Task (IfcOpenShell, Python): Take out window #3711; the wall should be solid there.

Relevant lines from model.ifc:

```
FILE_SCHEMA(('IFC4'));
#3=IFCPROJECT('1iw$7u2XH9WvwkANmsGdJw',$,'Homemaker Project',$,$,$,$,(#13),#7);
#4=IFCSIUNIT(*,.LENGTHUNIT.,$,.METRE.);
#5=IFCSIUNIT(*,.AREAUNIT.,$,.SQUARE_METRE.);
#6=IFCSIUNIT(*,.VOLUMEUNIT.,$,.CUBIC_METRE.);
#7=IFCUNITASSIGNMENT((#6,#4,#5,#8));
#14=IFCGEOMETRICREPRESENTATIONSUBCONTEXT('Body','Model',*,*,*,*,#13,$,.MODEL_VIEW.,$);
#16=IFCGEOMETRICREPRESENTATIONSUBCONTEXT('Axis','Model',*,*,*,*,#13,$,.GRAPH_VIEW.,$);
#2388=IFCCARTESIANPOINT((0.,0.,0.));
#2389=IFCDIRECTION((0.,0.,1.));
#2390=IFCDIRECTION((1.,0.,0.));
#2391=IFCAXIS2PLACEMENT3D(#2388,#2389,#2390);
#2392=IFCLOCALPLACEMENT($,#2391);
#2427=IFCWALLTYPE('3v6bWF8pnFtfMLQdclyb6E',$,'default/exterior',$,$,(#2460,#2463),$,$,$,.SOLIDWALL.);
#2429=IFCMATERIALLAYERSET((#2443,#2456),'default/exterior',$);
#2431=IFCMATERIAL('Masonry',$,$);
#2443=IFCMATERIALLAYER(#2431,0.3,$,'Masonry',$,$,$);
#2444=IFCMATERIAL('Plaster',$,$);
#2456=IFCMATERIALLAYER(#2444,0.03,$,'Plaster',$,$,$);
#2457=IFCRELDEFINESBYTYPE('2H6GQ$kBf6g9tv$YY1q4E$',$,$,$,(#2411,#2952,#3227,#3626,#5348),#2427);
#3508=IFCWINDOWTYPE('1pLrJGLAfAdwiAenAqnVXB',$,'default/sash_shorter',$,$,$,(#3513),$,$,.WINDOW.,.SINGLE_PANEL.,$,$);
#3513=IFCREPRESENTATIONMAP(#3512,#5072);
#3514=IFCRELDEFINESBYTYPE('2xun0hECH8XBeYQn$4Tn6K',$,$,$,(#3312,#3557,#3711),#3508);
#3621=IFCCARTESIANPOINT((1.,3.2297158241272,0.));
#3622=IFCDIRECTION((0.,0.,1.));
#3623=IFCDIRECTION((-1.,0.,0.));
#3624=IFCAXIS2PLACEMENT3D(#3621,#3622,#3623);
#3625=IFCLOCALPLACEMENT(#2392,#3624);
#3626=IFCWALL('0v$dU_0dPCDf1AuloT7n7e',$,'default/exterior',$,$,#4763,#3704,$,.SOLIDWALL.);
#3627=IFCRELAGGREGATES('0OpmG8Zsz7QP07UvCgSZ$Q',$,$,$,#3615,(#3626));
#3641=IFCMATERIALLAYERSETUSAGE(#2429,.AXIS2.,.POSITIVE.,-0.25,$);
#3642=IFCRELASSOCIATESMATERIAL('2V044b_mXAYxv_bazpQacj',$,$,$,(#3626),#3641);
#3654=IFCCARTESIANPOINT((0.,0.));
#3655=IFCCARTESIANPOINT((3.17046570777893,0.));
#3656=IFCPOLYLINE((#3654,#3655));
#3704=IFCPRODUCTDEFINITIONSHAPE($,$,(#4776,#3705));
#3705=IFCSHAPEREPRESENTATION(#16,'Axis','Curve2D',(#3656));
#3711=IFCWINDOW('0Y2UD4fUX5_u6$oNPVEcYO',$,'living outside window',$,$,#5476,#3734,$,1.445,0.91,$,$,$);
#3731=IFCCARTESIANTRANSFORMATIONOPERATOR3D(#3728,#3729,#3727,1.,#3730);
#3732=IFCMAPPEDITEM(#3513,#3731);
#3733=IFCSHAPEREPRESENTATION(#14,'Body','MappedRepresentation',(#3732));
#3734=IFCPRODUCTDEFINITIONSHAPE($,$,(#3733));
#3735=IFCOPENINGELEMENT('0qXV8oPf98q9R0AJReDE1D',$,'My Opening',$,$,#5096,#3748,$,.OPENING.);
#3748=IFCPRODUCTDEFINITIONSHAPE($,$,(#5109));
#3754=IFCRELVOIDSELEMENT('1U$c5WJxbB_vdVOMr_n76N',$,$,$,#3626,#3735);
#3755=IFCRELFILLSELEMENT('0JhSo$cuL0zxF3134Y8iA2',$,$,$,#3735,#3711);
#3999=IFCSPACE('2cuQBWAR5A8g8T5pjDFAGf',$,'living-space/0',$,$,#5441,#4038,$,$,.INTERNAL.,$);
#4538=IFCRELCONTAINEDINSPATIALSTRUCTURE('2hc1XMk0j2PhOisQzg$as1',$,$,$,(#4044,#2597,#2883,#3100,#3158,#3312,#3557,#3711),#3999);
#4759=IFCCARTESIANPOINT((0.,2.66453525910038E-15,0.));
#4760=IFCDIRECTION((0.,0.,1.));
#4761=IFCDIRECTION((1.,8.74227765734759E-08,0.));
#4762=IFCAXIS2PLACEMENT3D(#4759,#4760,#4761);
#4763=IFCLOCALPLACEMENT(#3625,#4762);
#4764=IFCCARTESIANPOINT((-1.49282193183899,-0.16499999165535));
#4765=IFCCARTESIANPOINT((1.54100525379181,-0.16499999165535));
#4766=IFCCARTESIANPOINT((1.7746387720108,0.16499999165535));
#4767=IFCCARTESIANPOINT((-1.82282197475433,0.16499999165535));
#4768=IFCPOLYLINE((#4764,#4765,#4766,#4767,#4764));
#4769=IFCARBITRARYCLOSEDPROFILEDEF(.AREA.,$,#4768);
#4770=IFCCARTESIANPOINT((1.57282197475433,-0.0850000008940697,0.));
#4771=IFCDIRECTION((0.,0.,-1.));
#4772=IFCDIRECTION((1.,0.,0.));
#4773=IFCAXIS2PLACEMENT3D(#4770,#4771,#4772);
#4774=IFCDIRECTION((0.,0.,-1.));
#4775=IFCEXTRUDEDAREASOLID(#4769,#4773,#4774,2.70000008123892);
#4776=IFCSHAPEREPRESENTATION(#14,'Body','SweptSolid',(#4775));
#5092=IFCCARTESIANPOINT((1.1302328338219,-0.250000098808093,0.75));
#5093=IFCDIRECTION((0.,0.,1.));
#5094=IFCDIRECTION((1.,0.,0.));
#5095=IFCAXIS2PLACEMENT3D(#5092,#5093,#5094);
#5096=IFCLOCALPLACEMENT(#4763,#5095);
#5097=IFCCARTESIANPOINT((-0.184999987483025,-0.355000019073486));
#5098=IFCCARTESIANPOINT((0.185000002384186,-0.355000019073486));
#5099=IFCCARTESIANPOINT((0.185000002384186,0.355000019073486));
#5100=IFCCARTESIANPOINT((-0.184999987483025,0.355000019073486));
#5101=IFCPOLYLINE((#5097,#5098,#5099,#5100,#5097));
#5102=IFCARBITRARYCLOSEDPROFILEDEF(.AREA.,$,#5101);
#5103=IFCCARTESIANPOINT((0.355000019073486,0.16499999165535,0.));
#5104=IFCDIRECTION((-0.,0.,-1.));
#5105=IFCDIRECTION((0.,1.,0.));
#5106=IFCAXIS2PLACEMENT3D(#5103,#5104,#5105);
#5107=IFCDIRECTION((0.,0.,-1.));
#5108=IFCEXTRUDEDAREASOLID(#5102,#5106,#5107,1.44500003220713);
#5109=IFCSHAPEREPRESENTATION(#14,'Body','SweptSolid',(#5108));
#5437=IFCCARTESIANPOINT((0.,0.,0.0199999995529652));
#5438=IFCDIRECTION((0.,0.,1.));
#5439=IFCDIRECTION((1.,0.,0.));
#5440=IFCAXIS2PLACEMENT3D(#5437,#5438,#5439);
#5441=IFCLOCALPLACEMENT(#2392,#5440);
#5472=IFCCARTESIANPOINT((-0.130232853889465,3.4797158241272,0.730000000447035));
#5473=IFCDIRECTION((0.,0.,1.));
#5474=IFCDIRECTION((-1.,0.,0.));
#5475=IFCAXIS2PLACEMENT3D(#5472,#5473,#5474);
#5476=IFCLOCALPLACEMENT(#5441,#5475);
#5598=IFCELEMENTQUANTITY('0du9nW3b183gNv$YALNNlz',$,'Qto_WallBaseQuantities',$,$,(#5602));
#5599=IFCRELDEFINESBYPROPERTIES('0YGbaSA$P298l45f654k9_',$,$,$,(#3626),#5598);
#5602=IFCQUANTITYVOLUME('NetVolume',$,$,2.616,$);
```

```python
import ifcopenshell
import ifcopenshell.api.feature
import ifcopenshell.api.pset
import ifcopenshell.api.root
import ifcopenshell.geom
import ifcopenshell.util.element
import ifcopenshell.util.shape
import ifcopenshell.util.unit

model = ifcopenshell.open("model.ifc")
volume_scale = ifcopenshell.util.unit.calculate_unit_scale(model, "VOLUMEUNIT")
settings = ifcopenshell.geom.settings()


def volume(element):
    """Net volume in cubic metres, openings subtracted."""
    shape = ifcopenshell.geom.create_shape(settings, element)
    return ifcopenshell.util.shape.get_volume(shape.geometry)


window = model.by_id(3711)
opening = window.FillsVoids[0].RelatingOpeningElement
wall = opening.VoidsElements[0].RelatingBuildingElement
before = volume(wall)

ifcopenshell.api.root.remove_product(model, product=window)
ifcopenshell.api.feature.remove_feature(model, feature=opening)

after = volume(wall)

# Update the wall's stored quantities.
qto = model.by_id(ifcopenshell.util.element.get_pset(wall, "Qto_WallBaseQuantities", should_inherit=False)["id"])
ifcopenshell.api.pset.edit_qto(model, qto=qto, properties={"NetVolume": after / volume_scale})

print(f"wall volume {before:.3f} -> {after:.3f} m3")

model.write("model_v2.ifc")
```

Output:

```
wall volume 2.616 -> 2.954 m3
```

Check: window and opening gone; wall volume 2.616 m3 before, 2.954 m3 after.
